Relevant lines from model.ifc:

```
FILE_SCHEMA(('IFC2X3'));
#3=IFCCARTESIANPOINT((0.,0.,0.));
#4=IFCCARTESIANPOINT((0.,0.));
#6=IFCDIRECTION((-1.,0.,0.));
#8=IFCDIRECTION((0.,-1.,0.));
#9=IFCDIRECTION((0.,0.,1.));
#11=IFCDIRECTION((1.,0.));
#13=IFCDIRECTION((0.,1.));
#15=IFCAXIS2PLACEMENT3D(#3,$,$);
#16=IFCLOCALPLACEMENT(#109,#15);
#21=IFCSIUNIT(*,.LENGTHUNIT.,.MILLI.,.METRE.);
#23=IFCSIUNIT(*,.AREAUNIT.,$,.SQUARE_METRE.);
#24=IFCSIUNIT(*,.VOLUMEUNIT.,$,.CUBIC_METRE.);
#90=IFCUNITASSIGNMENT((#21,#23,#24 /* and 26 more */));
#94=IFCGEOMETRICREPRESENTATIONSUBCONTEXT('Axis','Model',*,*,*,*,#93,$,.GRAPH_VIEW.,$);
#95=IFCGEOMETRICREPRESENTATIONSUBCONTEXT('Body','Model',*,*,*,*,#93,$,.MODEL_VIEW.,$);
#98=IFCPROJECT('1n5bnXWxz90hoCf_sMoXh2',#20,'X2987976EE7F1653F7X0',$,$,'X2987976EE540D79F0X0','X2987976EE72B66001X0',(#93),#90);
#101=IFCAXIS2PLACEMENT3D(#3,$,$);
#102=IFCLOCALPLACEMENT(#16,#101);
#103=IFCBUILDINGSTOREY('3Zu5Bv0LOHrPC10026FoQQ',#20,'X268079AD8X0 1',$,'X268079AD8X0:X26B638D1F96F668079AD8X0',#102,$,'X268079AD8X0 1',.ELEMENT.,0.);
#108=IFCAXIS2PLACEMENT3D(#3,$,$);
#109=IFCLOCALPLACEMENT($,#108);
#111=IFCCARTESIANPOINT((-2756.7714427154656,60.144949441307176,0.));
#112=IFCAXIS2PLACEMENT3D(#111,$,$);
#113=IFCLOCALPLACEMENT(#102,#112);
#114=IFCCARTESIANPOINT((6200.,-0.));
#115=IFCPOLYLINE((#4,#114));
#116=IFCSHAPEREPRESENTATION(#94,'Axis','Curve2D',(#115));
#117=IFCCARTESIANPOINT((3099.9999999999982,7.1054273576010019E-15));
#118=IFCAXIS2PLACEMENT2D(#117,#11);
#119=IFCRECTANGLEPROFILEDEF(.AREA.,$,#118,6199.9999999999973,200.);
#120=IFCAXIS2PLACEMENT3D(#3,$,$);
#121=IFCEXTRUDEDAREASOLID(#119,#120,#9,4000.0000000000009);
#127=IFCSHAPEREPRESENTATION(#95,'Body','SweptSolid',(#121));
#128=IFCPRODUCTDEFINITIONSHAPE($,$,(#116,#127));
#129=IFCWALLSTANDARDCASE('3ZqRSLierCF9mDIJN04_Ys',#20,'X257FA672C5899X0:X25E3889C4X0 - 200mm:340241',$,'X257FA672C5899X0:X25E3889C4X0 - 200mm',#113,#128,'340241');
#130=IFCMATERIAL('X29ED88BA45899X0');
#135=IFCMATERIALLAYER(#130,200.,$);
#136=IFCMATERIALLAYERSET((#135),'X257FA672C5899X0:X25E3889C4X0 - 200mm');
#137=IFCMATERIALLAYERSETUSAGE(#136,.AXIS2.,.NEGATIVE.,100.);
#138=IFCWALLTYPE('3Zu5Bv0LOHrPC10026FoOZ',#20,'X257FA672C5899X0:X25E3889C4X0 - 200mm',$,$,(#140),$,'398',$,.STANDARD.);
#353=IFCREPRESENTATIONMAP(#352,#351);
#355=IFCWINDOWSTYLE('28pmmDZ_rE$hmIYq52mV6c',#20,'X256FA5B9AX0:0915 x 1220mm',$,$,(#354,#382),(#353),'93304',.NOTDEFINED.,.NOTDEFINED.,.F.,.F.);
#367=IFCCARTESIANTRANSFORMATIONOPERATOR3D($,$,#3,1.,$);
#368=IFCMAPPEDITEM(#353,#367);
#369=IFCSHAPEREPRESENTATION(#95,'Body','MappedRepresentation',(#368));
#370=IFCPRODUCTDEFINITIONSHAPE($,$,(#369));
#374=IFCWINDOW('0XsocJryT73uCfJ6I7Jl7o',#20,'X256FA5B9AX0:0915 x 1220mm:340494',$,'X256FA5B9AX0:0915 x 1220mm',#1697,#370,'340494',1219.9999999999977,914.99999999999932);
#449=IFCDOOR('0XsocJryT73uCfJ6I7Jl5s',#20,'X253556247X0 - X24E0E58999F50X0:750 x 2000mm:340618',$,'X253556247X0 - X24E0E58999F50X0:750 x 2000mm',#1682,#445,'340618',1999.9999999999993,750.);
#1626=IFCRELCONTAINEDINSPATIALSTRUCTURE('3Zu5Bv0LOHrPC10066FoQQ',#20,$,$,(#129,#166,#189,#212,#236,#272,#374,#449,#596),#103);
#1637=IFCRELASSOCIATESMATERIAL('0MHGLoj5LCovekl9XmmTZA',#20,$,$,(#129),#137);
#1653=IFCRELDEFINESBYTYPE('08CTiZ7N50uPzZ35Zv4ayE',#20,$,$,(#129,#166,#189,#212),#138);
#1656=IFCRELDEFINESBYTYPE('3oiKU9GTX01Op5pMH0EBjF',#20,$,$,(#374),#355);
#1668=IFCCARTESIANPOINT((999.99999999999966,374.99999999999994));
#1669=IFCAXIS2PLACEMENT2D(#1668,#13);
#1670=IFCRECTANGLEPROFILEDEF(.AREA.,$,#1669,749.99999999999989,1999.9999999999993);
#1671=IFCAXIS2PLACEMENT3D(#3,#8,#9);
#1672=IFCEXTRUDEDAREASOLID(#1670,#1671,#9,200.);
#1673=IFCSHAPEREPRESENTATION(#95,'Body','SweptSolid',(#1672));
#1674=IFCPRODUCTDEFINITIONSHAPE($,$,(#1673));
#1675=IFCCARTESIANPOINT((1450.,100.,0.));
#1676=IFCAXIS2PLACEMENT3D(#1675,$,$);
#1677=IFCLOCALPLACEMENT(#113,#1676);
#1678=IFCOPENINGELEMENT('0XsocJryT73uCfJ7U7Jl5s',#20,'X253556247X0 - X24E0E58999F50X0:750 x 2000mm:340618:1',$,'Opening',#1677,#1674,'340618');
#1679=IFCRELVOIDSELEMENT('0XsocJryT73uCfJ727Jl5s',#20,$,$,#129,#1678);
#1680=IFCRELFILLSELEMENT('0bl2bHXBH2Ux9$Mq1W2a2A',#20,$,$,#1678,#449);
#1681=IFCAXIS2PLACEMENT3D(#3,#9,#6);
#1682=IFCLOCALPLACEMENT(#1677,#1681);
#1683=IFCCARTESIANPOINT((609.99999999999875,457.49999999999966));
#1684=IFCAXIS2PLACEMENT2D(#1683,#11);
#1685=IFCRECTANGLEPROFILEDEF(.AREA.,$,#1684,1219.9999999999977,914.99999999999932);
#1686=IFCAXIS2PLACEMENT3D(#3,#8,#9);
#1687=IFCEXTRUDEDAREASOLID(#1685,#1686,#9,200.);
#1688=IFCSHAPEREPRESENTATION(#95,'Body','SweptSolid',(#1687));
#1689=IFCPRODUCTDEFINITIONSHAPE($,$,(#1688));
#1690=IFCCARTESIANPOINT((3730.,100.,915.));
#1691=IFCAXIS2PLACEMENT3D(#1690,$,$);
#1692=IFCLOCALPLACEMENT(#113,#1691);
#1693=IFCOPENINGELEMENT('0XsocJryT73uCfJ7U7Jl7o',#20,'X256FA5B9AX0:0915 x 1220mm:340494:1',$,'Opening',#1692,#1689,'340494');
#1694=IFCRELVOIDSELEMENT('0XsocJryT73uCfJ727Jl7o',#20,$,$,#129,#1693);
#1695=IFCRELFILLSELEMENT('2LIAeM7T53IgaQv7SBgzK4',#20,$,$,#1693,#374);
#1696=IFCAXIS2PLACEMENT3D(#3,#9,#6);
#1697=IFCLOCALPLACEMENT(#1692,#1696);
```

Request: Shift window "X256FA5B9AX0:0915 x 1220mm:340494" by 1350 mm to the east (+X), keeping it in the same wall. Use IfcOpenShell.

```python
import ifcopenshell
import ifcopenshell.api.geometry
import ifcopenshell.util.placement
import ifcopenshell.util.unit

model = ifcopenshell.open("model.ifc")
unit_scale = ifcopenshell.util.unit.calculate_unit_scale(model)

window = model.by_id(374)
opening = window.FillsVoids[0].RelatingOpeningElement
wall = opening.VoidsElements[0].RelatingBuildingElement

wall_matrix = ifcopenshell.util.placement.get_local_placement(wall.ObjectPlacement)
shift = wall_matrix[:3, 0] * 1.35 / unit_scale
before = ifcopenshell.util.placement.get_local_placement(window.ObjectPlacement)[:3, 3].copy()

# The window is placed relative to its opening, so it follows when the opening moves.
matrix = ifcopenshell.util.placement.get_local_placement(opening.ObjectPlacement)
matrix[:3, 3] += shift
ifcopenshell.api.geometry.edit_object_placement(
    model, product=opening, matrix=matrix, is_si=False, should_transform_children=True
)

after = ifcopenshell.util.placement.get_local_placement(window.ObjectPlacement)[:3, 3]
print("window moved by", (after - before).round(3) + 0.0)

model.write("model_rev.ifc")
```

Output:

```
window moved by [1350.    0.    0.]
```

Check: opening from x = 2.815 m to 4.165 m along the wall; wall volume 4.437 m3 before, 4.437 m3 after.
